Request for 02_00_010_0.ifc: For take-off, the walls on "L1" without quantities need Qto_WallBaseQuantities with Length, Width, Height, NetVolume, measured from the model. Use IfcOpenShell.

First a look at what the model holds.

```python
import ifcopenshell
import ifcopenshell.util.element
import ifcopenshell.util.unit

model = ifcopenshell.open("02_00_010_0.ifc")
print(model.schema)
for unit_type in ("LENGTHUNIT", "AREAUNIT", "VOLUMEUNIT"):
    print(unit_type, ifcopenshell.util.unit.calculate_unit_scale(model, unit_type))
storey = next(s for s in model.by_type("IfcBuildingStorey") if s.Name == "L1")
walls = [e for e in ifcopenshell.util.element.get_decomposition(storey) if e.is_a("IfcWall")]
for e in sorted(walls, key=lambda e: e.id()):
    print(e.id(), e.is_a(), e.Name, list(ifcopenshell.util.element.get_psets(e, qtos_only=True)), sep=" | ")
```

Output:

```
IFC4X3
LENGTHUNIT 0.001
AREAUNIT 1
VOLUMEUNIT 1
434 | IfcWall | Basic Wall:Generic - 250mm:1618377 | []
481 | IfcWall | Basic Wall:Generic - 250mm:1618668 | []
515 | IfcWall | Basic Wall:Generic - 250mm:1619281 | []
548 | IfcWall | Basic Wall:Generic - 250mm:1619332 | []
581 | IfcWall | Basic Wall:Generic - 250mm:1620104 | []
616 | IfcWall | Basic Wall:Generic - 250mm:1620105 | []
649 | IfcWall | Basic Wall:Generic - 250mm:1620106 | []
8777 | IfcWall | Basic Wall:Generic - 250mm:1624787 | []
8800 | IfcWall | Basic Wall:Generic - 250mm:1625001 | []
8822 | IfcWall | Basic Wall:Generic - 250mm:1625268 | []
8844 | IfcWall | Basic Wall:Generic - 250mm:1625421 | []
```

```python
import ifcopenshell
import ifcopenshell.api.pset
import ifcopenshell.geom
import ifcopenshell.util.element
import ifcopenshell.util.shape
import ifcopenshell.util.unit

model = ifcopenshell.open("02_00_010_0.ifc")
unit_scale = ifcopenshell.util.unit.calculate_unit_scale(model)
volume_scale = ifcopenshell.util.unit.calculate_unit_scale(model, "VOLUMEUNIT")
settings = ifcopenshell.geom.settings()

storey = next(s for s in model.by_type("IfcBuildingStorey") if s.Name == "L1")
walls = [e for e in ifcopenshell.util.element.get_decomposition(storey) if e.is_a("IfcWall")]

for e in sorted(walls, key=lambda e: e.id()):
    if ifcopenshell.util.element.get_psets(e, qtos_only=True, should_inherit=False):
        continue
    # Geometry comes back in metres, in the element's own axes.
    shape = ifcopenshell.geom.create_shape(settings, e)
    values = {
        "Length": ifcopenshell.util.shape.get_x(shape.geometry) / unit_scale,
        "Width": ifcopenshell.util.shape.get_y(shape.geometry) / unit_scale,
        "Height": ifcopenshell.util.shape.get_z(shape.geometry) / unit_scale,
        "NetVolume": ifcopenshell.util.shape.get_volume(shape.geometry) / volume_scale,
    }
    qto = ifcopenshell.api.pset.add_qto(model, product=e, name="Qto_WallBaseQuantities")
    ifcopenshell.api.pset.edit_qto(model, qto=qto, properties=values)
    print(e.id(), {k: round(v, 3) for k, v in values.items()})

model.write("02_00_010_0_v2.ifc")
```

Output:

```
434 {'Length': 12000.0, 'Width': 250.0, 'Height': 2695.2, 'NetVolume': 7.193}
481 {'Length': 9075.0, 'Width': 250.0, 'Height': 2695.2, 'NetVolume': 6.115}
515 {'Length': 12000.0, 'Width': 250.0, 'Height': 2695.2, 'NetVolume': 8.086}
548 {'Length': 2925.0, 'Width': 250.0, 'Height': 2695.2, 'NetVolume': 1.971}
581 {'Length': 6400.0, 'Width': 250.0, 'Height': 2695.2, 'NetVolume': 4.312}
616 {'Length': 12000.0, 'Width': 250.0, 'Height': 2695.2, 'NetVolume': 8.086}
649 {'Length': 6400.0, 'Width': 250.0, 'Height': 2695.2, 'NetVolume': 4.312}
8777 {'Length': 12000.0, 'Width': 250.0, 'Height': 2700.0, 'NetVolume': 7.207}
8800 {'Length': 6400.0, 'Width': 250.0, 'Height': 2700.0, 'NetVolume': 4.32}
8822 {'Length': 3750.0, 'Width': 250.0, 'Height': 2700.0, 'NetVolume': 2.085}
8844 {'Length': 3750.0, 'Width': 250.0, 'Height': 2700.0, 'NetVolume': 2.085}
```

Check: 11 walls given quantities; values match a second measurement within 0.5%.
